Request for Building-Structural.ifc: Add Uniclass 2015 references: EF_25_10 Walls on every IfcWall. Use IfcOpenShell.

First a look at what the model holds.

```python
import ifcopenshell

model = ifcopenshell.open("Building-Structural.ifc")
print(model.schema)
print("classifications:", [c.Name for c in model.by_type("IfcClassification")])
for ifc_class in ("IfcDoor", "IfcRoof", "IfcStair", "IfcWall", "IfcWindow"):
    print(ifc_class, len(model.by_type(ifc_class)))
```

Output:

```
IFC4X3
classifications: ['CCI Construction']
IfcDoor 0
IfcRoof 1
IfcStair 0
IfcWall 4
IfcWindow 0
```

```python
import ifcopenshell
import ifcopenshell.api.classification

model = ifcopenshell.open("Building-Structural.ifc")

system = ifcopenshell.api.classification.add_classification(model, classification="Uniclass 2015")

codes = {
    "IfcWall": ("EF_25_10", "Walls"),
}
for ifc_class, (code, name) in codes.items():
    products = model.by_type(ifc_class)
    ifcopenshell.api.classification.add_reference(
        model, products=products, classification=system, identification=code, name=name
    )
    print(code, len(products))

model.write("Building-Structural_v2.ifc")
```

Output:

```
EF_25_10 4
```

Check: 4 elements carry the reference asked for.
